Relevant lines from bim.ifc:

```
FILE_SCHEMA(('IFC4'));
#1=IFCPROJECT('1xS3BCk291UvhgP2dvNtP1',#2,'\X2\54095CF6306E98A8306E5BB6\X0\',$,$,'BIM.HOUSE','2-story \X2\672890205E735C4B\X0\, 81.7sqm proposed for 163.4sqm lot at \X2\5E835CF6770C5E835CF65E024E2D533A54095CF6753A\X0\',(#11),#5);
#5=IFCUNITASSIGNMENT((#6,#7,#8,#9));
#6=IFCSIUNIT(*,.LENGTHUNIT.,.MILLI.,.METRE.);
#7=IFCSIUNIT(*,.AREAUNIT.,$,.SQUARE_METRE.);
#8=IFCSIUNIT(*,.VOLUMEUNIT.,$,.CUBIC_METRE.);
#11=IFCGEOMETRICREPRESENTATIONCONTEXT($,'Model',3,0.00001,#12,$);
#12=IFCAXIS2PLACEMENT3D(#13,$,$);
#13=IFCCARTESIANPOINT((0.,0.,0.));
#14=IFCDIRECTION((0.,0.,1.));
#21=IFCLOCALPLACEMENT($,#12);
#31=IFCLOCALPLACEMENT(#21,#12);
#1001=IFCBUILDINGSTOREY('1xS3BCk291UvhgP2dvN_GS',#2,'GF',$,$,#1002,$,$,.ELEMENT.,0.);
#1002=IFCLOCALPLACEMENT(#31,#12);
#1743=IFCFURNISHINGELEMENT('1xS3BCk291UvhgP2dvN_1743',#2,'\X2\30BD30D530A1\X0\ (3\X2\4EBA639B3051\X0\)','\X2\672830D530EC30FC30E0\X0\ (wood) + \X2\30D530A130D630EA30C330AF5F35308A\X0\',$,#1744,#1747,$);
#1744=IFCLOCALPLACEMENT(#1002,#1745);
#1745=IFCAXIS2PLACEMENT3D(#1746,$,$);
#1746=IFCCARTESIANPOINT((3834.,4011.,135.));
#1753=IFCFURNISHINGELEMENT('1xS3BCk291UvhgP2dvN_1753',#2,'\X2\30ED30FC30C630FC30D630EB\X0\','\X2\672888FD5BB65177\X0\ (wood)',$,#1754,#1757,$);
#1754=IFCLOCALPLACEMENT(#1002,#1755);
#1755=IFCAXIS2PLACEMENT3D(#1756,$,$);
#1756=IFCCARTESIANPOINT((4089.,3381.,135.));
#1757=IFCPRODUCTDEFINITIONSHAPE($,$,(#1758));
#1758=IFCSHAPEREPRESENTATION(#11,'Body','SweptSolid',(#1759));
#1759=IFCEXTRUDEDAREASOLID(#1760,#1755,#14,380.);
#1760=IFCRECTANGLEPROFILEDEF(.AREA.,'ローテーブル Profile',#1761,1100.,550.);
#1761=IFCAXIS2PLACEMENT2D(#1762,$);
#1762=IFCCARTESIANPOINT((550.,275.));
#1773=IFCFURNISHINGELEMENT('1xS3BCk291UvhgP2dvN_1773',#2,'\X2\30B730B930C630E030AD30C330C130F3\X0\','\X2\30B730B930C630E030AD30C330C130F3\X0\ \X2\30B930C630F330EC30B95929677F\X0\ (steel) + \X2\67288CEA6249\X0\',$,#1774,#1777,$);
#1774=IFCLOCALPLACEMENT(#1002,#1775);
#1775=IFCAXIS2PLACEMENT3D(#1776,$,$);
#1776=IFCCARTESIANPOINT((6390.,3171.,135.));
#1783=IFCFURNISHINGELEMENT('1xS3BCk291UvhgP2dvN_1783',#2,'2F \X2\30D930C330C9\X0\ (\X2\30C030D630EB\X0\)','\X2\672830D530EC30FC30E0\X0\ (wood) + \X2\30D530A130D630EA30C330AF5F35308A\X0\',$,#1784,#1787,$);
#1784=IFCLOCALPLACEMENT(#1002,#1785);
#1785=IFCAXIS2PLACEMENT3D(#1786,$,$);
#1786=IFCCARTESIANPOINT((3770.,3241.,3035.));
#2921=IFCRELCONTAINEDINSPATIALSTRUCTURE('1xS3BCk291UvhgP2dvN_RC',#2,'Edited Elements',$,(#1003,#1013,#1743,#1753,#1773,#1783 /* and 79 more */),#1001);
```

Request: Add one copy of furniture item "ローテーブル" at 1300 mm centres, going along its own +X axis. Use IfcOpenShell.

```python
import ifcopenshell
import ifcopenshell.api.geometry
import ifcopenshell.api.root
import ifcopenshell.util.element
import ifcopenshell.util.placement

model = ifcopenshell.open("bim.ifc")


def reuse_history(source, copy):
    """copy_class also copies each property set's owner history, people and application; keep the originals."""
    for rel in copy.IsDefinedBy:
        if rel.is_a("IfcRelDefinesByProperties") and (history := rel.RelatingPropertyDefinition.OwnerHistory):
            rel.RelatingPropertyDefinition.OwnerHistory = source.OwnerHistory
            ifcopenshell.util.element.remove_deep2(model, history)


source = model.by_guid("1xS3BCk291UvhgP2dvN_1753")
base = ifcopenshell.util.placement.get_local_placement(source.ObjectPlacement)
step = base[:3, 0] * 1300.0

for i in range(1, 2):
    copy = ifcopenshell.api.root.copy_class(model, product=source)
    copy.Representation = ifcopenshell.util.element.copy_deep(
        model, source.Representation, exclude=["IfcGeometricRepresentationContext", "IfcRepresentationMap"]
    )
    reuse_history(source, copy)
    matrix = base.copy()
    matrix[:3, 3] += i * step
    print("added at", matrix[:3, 3].round(3) + 0.0)
    ifcopenshell.api.geometry.edit_object_placement(model, product=copy, matrix=matrix, is_si=False)

model.write("bim-out.ifc")
```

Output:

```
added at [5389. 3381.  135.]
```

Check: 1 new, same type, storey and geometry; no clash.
